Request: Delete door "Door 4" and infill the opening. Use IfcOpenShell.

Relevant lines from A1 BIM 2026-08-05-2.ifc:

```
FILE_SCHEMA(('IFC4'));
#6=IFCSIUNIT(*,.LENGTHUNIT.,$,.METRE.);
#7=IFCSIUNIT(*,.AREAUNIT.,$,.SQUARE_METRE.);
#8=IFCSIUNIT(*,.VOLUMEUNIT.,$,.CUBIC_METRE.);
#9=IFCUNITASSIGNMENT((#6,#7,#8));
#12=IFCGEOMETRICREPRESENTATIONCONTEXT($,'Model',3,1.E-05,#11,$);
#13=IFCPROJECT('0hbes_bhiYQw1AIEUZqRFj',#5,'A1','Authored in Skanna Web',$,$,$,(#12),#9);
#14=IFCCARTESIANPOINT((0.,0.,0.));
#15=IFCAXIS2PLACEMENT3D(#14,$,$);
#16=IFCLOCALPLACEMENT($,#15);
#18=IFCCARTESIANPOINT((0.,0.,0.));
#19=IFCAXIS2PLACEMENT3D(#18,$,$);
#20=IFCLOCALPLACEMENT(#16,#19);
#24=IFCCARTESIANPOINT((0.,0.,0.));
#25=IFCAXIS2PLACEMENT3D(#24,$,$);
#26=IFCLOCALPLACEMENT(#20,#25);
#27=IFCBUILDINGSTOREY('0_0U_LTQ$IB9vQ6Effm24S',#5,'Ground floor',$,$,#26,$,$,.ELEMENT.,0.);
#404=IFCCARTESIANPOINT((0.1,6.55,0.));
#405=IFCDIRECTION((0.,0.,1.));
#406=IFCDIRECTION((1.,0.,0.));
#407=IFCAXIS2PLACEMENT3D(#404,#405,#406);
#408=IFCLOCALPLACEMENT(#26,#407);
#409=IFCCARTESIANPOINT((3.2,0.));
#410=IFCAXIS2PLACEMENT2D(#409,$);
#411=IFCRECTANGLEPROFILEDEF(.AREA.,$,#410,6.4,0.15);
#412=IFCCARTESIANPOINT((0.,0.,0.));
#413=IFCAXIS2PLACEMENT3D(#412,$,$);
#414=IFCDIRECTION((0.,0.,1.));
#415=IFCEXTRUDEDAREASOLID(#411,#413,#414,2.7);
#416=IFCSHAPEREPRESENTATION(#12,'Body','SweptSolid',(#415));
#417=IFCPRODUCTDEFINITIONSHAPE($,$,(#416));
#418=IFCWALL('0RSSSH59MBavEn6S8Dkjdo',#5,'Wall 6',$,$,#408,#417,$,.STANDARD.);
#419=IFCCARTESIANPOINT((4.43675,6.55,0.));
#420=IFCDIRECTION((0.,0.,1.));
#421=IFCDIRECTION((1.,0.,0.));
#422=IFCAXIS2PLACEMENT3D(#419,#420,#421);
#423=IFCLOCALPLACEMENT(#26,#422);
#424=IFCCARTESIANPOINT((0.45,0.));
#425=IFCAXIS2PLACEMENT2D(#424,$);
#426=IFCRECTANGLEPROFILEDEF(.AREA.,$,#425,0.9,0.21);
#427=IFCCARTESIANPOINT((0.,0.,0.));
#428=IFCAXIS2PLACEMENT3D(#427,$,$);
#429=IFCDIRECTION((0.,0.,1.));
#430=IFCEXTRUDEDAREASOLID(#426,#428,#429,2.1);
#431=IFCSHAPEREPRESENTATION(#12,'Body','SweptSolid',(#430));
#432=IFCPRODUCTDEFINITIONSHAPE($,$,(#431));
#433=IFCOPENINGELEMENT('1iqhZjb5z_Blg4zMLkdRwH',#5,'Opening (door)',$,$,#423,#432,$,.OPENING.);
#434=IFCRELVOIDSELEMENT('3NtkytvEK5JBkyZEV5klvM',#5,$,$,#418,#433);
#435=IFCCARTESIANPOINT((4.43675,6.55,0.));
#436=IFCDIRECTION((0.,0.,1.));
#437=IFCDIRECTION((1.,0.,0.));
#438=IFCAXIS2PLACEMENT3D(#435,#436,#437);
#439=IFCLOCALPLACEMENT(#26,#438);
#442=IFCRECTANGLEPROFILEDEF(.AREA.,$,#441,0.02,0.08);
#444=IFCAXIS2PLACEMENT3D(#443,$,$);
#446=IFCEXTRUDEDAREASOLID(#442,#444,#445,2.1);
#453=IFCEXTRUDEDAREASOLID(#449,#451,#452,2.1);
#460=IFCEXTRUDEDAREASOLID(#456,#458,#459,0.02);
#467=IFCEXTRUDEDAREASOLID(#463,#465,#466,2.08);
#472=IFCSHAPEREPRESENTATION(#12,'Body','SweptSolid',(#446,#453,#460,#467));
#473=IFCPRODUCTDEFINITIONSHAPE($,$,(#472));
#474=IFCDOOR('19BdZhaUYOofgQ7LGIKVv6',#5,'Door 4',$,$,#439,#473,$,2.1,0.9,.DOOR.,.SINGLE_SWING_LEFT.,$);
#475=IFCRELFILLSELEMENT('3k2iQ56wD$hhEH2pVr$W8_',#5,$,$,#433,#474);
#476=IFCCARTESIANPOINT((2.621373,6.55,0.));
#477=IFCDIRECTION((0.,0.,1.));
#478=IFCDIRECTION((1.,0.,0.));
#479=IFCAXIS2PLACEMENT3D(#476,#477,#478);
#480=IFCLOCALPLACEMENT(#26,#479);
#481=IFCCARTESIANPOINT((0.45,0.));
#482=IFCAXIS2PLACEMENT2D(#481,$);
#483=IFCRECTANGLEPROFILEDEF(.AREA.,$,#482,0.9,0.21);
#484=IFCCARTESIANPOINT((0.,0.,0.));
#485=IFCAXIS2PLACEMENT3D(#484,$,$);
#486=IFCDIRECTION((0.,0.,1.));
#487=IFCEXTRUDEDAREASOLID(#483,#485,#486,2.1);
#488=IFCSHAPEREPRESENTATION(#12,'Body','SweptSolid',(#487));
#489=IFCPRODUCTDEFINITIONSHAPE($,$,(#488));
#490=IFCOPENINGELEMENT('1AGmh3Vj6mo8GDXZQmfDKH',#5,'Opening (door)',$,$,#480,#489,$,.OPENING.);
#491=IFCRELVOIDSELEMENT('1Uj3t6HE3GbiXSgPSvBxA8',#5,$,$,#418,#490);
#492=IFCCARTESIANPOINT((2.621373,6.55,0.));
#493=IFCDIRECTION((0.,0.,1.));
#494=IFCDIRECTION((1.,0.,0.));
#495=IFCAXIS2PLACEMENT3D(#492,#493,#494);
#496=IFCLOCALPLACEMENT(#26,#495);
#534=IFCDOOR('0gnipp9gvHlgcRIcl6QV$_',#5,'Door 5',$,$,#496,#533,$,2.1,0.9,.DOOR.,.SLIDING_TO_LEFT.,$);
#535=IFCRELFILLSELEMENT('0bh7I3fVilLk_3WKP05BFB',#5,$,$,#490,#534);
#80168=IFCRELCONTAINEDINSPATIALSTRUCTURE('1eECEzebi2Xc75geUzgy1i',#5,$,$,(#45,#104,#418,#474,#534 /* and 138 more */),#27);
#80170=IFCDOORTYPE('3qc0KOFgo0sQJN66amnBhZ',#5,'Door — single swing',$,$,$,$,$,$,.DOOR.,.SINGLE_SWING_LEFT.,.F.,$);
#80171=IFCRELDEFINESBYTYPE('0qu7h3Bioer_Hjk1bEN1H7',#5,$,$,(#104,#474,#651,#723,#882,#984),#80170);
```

```python
import ifcopenshell
import ifcopenshell.api.feature
import ifcopenshell.api.root
import ifcopenshell.geom
import ifcopenshell.util.shape

model = ifcopenshell.open("A1 BIM 2026-08-05-2.ifc")
settings = ifcopenshell.geom.settings()


def volume(element):
    """Net volume in cubic metres, openings subtracted."""
    shape = ifcopenshell.geom.create_shape(settings, element)
    return ifcopenshell.util.shape.get_volume(shape.geometry)


door = model.by_guid("19BdZhaUYOofgQ7LGIKVv6")
opening = door.FillsVoids[0].RelatingOpeningElement
wall = opening.VoidsElements[0].RelatingBuildingElement
before = volume(wall)

ifcopenshell.api.root.remove_product(model, product=door)
ifcopenshell.api.feature.remove_feature(model, feature=opening)

after = volume(wall)

print(f"wall volume {before:.3f} -> {after:.3f} m3")

model.write("A1 BIM 2026-08-05-2_rev.ifc")
```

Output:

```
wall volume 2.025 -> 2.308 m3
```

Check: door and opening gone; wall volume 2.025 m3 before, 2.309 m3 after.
